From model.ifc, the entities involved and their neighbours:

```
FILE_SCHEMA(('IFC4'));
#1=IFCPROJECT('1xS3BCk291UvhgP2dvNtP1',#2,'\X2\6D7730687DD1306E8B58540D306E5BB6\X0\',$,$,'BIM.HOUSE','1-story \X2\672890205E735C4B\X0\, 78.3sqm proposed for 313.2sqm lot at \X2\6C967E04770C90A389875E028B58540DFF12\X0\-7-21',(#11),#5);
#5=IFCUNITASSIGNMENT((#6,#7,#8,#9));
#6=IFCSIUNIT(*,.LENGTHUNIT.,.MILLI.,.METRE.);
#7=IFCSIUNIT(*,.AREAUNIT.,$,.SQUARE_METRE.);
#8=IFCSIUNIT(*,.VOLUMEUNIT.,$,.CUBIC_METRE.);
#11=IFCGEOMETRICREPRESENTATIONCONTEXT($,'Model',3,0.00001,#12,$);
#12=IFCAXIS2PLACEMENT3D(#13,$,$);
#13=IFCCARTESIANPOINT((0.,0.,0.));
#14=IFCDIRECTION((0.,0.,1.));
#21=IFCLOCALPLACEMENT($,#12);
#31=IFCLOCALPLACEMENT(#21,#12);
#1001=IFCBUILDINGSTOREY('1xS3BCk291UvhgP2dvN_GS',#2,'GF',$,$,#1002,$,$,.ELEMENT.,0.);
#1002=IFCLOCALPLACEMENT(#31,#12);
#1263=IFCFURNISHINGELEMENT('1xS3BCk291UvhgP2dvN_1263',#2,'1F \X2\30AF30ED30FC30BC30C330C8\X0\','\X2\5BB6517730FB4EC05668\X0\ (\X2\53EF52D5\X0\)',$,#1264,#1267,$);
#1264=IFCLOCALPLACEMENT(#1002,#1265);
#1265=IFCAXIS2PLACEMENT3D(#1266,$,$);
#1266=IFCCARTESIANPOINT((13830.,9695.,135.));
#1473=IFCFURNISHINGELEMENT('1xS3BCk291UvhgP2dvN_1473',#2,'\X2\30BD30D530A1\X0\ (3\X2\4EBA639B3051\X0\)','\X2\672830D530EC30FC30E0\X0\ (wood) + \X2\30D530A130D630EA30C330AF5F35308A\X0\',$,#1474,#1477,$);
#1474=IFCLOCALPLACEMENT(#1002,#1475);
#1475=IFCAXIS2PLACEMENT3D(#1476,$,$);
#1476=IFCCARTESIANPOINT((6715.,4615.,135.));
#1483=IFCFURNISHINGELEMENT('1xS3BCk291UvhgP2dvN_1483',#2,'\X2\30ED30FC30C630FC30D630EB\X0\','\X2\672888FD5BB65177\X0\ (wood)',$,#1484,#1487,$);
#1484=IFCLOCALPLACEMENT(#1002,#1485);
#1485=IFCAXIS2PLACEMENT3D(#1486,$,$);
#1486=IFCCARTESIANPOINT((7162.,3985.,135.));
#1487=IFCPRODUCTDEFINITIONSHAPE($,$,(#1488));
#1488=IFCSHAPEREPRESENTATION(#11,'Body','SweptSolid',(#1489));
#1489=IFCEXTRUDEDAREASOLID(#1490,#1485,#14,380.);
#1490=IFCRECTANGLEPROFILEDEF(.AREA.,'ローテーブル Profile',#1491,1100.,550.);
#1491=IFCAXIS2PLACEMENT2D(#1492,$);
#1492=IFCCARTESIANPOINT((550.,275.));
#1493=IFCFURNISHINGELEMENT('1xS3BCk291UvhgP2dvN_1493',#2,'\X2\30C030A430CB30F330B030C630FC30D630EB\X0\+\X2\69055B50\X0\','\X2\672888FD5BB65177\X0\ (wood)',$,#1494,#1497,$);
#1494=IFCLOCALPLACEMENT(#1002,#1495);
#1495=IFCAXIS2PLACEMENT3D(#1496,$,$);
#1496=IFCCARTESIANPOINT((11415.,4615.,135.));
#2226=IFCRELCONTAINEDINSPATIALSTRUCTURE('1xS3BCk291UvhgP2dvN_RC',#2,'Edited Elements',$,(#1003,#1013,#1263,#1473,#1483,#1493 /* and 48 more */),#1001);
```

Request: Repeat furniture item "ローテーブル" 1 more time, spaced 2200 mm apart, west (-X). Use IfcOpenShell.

```python
import numpy as np
import ifcopenshell
import ifcopenshell.api.geometry
import ifcopenshell.api.root
import ifcopenshell.util.element
import ifcopenshell.util.placement
import ifcopenshell.util.unit

model = ifcopenshell.open("model.ifc")
unit_scale = ifcopenshell.util.unit.calculate_unit_scale(model)


def reuse_history(source, copy):
    """copy_class also copies each property set's owner history, people and application; keep the originals."""
    for rel in copy.IsDefinedBy:
        if rel.is_a("IfcRelDefinesByProperties") and (history := rel.RelatingPropertyDefinition.OwnerHistory):
            rel.RelatingPropertyDefinition.OwnerHistory = source.OwnerHistory
            ifcopenshell.util.element.remove_deep2(model, history)


source = model.by_guid("1xS3BCk291UvhgP2dvN_1483")
base = ifcopenshell.util.placement.get_local_placement(source.ObjectPlacement)
step = np.array([-1.0, 0.0, 0.0]) * 2.2 / unit_scale

for i in range(1, 2):
    copy = ifcopenshell.api.root.copy_class(model, product=source)
    copy.Representation = ifcopenshell.util.element.copy_deep(
        model, source.Representation, exclude=["IfcGeometricRepresentationContext", "IfcRepresentationMap"]
    )
    reuse_history(source, copy)
    matrix = base.copy()
    matrix[:3, 3] += i * step
    print("added at", matrix[:3, 3].round(3) + 0.0)
    ifcopenshell.api.geometry.edit_object_placement(model, product=copy, matrix=matrix, is_si=False)

model.write("model-out.ifc")
```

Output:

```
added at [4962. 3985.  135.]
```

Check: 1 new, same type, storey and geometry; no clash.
